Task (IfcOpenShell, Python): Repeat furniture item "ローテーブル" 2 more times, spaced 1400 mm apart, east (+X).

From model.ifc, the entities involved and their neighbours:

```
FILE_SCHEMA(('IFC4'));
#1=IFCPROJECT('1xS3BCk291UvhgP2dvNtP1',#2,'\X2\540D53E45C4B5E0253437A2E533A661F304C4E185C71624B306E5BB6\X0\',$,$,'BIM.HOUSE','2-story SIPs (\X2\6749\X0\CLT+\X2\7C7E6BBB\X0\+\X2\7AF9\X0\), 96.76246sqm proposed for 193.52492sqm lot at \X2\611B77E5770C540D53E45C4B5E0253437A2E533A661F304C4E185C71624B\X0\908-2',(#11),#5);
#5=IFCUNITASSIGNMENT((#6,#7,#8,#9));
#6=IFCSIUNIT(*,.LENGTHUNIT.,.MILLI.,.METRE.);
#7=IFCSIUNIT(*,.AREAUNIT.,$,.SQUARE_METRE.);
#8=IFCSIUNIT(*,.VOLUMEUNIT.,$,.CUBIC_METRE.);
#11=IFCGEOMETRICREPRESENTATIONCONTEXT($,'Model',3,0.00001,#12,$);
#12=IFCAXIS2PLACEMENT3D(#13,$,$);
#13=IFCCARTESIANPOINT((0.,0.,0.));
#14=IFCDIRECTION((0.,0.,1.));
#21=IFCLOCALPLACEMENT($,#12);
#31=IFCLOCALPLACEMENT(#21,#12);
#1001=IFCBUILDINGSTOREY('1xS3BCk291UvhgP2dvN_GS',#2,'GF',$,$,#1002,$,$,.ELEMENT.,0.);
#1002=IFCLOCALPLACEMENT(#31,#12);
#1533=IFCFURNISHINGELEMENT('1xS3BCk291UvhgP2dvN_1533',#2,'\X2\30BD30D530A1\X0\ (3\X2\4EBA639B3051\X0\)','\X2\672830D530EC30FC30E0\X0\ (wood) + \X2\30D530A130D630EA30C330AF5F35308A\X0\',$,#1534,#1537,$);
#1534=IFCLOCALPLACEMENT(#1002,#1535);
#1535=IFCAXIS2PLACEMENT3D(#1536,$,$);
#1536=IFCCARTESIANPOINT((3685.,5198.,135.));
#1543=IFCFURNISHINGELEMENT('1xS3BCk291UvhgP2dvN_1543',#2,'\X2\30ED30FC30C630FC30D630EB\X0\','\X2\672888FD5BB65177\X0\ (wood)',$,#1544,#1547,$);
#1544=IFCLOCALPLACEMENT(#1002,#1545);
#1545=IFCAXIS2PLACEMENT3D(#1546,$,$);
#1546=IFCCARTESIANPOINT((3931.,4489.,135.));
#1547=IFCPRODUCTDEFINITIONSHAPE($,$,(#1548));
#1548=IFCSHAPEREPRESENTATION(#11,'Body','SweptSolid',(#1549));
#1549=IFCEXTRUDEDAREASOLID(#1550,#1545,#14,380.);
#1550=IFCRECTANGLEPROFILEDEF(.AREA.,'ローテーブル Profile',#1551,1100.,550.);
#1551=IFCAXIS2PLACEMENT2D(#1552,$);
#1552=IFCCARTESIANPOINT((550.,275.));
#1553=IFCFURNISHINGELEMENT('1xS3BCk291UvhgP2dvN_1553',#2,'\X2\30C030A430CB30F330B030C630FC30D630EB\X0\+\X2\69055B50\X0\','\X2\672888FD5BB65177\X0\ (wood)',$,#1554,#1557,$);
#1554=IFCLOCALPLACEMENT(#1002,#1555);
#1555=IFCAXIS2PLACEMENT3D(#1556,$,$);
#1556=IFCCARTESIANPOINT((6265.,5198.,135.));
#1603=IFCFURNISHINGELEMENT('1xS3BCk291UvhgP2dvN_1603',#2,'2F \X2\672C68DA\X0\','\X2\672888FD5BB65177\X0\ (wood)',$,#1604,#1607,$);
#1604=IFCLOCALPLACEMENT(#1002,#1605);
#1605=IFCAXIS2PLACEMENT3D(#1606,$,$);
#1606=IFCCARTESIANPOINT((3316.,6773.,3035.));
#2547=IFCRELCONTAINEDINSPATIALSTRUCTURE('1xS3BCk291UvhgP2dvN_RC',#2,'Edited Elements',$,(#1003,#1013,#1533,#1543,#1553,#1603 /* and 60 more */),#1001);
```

```python
import numpy as np
import ifcopenshell
import ifcopenshell.api.geometry
import ifcopenshell.api.root
import ifcopenshell.util.element
import ifcopenshell.util.placement

model = ifcopenshell.open("model.ifc")


def reuse_history(source, copy):
    """copy_class also copies each property set's owner history, people and application; keep the originals."""
    for rel in copy.IsDefinedBy:
        if rel.is_a("IfcRelDefinesByProperties") and (history := rel.RelatingPropertyDefinition.OwnerHistory):
            rel.RelatingPropertyDefinition.OwnerHistory = source.OwnerHistory
            ifcopenshell.util.element.remove_deep2(model, history)


source = model.by_guid("1xS3BCk291UvhgP2dvN_1543")
base = ifcopenshell.util.placement.get_local_placement(source.ObjectPlacement)
step = np.array([1.0, 0.0, 0.0]) * 1400.0

for i in range(1, 3):
    copy = ifcopenshell.api.root.copy_class(model, product=source)
    copy.Representation = ifcopenshell.util.element.copy_deep(
        model, source.Representation, exclude=["IfcGeometricRepresentationContext", "IfcRepresentationMap"]
    )
    reuse_history(source, copy)
    matrix = base.copy()
    matrix[:3, 3] += i * step
    print("added at", matrix[:3, 3].round(3) + 0.0)
    ifcopenshell.api.geometry.edit_object_placement(model, product=copy, matrix=matrix, is_si=False)

model.write("model-out.ifc")
```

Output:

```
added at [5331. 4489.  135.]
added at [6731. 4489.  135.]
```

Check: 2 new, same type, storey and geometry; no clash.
